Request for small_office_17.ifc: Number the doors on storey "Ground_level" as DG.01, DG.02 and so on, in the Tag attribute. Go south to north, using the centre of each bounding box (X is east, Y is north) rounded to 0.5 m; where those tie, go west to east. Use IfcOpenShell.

First a look at what the model holds.

```python
import ifcopenshell
import ifcopenshell.util.element
import ifcopenshell.util.placement

model = ifcopenshell.open("small_office_17.ifc")
print(model.schema)
storey = next(s for s in model.by_type("IfcBuildingStorey") if s.Name == "Ground_level")
doors = [e for e in ifcopenshell.util.element.get_decomposition(storey) if e.is_a("IfcDoor")]
for e in sorted(doors, key=lambda e: e.id()):
    origin = ifcopenshell.util.placement.get_local_placement(e.ObjectPlacement)[:3, 3]
    print(e.id(), e.Tag, e.Name, origin.round(2) + 0.0, sep=" | ")
```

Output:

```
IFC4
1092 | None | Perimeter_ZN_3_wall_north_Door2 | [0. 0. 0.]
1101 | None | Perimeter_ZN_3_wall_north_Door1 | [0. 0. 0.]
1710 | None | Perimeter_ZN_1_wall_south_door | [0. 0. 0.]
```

```python
import ifcopenshell
import ifcopenshell.geom
import ifcopenshell.util.element
import ifcopenshell.util.shape

model = ifcopenshell.open("small_office_17.ifc")
settings = ifcopenshell.geom.settings()
settings.set("use-world-coords", True)


def centre(element):
    shape = ifcopenshell.geom.create_shape(settings, element)
    return ifcopenshell.util.shape.get_bbox_centroid(shape.geometry)


storey = next(s for s in model.by_type("IfcBuildingStorey") if s.Name == "Ground_level")
doors = [e for e in ifcopenshell.util.element.get_decomposition(storey) if e.is_a("IfcDoor")]

# Insertion points can sit at a corner or the storey origin, so sort by the geometry (in metres).
centres = {e: centre(e) for e in doors}
doors.sort(key=lambda e: (round(centres[e][1] / 0.5), centres[e][0]))

for i, e in enumerate(doors, start=1):
    number = f"DG.{i:02d}"
    e.Tag = number
    print(e.id(), number)

model.write("small_office_17_updated.ifc")
```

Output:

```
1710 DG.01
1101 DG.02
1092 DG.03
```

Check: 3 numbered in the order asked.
